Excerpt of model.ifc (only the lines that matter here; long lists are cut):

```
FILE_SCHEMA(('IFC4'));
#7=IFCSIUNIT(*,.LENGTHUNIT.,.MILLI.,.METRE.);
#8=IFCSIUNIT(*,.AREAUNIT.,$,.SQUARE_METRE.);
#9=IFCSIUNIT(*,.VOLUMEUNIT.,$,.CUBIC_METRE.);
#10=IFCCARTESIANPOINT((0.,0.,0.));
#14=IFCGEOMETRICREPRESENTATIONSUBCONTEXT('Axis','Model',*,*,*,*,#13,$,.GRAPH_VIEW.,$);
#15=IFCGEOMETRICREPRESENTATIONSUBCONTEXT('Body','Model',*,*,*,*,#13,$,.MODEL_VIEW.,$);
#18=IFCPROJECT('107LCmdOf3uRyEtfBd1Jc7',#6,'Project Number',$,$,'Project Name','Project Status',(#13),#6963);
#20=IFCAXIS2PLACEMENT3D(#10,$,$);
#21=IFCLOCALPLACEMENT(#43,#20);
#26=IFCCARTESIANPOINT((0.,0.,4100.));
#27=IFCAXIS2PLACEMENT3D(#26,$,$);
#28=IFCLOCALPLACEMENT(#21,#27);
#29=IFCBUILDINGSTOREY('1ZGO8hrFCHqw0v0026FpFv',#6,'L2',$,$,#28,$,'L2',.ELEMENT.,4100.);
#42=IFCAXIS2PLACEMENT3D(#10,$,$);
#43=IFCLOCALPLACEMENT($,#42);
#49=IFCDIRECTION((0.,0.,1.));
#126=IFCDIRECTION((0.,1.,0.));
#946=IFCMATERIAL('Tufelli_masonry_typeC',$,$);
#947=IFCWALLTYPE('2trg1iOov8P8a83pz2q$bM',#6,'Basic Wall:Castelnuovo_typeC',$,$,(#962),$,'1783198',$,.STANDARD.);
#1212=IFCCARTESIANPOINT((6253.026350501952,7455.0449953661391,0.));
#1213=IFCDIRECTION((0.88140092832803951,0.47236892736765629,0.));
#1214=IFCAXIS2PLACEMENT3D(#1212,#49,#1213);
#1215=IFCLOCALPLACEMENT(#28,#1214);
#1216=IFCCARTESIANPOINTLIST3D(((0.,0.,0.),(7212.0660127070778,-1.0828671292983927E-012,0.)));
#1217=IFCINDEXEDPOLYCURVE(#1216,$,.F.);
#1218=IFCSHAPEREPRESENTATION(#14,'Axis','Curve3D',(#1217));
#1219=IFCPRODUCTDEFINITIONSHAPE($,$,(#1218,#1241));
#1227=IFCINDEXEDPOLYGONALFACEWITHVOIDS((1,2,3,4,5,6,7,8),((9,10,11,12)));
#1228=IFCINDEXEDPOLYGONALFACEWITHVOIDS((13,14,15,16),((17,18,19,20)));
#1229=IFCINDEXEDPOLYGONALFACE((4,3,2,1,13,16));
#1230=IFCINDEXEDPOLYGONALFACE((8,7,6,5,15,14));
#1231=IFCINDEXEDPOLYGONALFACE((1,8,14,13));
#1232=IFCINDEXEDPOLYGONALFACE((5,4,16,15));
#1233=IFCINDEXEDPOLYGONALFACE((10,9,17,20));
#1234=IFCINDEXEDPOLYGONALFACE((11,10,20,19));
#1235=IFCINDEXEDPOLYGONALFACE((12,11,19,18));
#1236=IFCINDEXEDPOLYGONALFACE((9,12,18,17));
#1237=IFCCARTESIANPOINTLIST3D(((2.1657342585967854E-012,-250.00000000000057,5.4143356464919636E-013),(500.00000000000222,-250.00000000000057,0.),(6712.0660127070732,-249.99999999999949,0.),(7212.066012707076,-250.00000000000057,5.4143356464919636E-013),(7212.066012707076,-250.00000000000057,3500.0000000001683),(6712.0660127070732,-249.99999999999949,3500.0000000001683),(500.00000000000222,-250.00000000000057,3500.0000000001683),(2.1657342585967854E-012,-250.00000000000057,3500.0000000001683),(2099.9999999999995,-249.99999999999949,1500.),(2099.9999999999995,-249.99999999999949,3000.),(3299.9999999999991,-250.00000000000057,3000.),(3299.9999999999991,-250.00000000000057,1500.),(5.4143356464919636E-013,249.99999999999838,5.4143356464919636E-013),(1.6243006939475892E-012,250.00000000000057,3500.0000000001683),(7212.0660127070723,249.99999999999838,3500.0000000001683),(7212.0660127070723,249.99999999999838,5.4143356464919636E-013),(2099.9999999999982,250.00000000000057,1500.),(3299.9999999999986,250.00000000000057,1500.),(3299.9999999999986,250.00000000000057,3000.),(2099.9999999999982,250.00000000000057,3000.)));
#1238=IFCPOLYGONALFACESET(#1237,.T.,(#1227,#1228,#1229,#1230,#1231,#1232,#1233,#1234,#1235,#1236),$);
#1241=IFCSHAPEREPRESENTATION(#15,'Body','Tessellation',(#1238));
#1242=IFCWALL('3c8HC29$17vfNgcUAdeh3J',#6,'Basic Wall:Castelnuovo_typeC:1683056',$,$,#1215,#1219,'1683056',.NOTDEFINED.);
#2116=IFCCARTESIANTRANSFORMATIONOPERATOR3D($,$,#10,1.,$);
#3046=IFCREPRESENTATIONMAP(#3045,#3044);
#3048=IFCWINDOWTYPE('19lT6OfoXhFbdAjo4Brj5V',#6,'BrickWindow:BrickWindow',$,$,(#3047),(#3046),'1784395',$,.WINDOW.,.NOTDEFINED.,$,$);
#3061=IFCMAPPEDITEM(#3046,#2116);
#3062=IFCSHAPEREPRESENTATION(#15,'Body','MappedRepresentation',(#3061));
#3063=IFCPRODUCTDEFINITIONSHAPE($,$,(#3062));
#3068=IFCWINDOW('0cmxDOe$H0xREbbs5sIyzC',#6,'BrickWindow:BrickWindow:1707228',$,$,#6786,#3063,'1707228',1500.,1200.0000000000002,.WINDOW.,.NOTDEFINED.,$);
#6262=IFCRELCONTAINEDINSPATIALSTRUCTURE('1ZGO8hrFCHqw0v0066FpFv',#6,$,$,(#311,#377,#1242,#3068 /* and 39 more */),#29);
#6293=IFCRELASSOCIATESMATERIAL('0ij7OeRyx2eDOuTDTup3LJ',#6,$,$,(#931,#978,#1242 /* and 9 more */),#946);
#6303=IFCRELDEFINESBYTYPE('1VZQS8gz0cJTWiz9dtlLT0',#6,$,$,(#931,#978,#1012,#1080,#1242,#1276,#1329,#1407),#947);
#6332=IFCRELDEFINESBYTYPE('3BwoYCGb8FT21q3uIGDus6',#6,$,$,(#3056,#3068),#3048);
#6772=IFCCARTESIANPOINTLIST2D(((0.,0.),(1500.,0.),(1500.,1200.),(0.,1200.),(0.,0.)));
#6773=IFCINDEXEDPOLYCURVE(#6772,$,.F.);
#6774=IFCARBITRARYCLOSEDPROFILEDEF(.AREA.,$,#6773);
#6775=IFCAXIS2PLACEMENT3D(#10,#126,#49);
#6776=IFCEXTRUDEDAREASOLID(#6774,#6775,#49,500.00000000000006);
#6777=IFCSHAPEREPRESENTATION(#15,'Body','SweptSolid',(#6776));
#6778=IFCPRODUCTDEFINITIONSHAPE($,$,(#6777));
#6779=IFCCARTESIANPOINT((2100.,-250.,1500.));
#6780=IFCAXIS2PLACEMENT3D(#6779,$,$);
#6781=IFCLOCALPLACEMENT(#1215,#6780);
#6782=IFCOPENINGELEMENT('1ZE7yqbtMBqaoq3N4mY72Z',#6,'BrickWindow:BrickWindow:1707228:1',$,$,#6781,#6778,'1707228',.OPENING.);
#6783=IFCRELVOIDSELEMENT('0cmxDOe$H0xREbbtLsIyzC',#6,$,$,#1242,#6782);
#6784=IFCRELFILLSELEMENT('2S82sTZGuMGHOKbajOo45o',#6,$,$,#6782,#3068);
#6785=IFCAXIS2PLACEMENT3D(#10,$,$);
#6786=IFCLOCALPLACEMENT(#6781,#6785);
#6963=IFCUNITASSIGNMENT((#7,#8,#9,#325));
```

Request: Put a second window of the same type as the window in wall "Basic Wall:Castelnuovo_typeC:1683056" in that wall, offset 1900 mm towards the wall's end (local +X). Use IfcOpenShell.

```python
import ifcopenshell
import ifcopenshell.api.feature
import ifcopenshell.api.geometry
import ifcopenshell.api.root
import ifcopenshell.geom
import ifcopenshell.util.element
import ifcopenshell.util.placement
import ifcopenshell.util.shape
import ifcopenshell.util.unit

model = ifcopenshell.open("model.ifc")
unit_scale = ifcopenshell.util.unit.calculate_unit_scale(model)
settings = ifcopenshell.geom.settings()


def volume(element):
    """Net volume in cubic metres, openings subtracted."""
    shape = ifcopenshell.geom.create_shape(settings, element)
    return ifcopenshell.util.shape.get_volume(shape.geometry)


def reuse_history(source, copy):
    """copy_class also copies each property set's owner history, people and application; keep the originals."""
    for rel in copy.IsDefinedBy:
        if rel.is_a("IfcRelDefinesByProperties") and (history := rel.RelatingPropertyDefinition.OwnerHistory):
            rel.RelatingPropertyDefinition.OwnerHistory = source.OwnerHistory
            ifcopenshell.util.element.remove_deep2(model, history)


window = model.by_id(3068)
opening = window.FillsVoids[0].RelatingOpeningElement
wall = opening.VoidsElements[0].RelatingBuildingElement
before = volume(wall)
shift = ifcopenshell.util.placement.get_local_placement(wall.ObjectPlacement)[:3, 0] * 1.9 / unit_scale

# copy_class copies the void relationship, type, container and properties, but no geometry.
new_opening = ifcopenshell.api.root.copy_class(model, product=opening)
new_opening.Representation = ifcopenshell.util.element.copy_deep(
    model, opening.Representation, exclude=["IfcGeometricRepresentationContext", "IfcRepresentationMap"]
)
new_opening.Name = "BrickWindow:BrickWindow"
new_opening.Tag = None
new_window = ifcopenshell.api.root.copy_class(model, product=window)
new_window.Representation = ifcopenshell.util.element.copy_deep(
    model, window.Representation, exclude=["IfcGeometricRepresentationContext", "IfcRepresentationMap"]
)
new_window.Name = "BrickWindow:BrickWindow"
new_window.Tag = None
reuse_history(window, new_window)
ifcopenshell.api.feature.add_filling(model, opening=new_opening, element=new_window)

for old, new in ((opening, new_opening), (window, new_window)):
    matrix = ifcopenshell.util.placement.get_local_placement(old.ObjectPlacement)
    matrix[:3, 3] += shift
    ifcopenshell.api.geometry.edit_object_placement(model, product=new, matrix=matrix, is_si=False)

after = volume(wall)

print(f"wall volume {before:.3f} -> {after:.3f} m3")

model.write("model_v2.ifc")
```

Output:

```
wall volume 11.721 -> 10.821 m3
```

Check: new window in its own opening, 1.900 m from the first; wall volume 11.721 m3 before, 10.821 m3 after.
